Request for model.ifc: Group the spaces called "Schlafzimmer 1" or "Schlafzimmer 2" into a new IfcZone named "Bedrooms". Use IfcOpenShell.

First a look at what the model holds.

```python
import ifcopenshell

model = ifcopenshell.open("model.ifc")
print(model.schema)
seen = {}
for space in model.by_type("IfcSpace"):
    seen[space.LongName] = seen.get(space.LongName, 0) + 1
for name, count in sorted(seen.items(), key=str):
    print(count, "x", name)
print("zones:", [z.Name for z in model.by_type("IfcZone")][:20])
```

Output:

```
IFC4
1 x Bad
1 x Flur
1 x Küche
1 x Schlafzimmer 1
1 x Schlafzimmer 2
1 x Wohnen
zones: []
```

```python
import ifcopenshell
import ifcopenshell.api.group
import ifcopenshell.api.root

model = ifcopenshell.open("model.ifc")

names = {"Schlafzimmer 1", "Schlafzimmer 2"}
spaces = [s for s in model.by_type("IfcSpace") if s.LongName in names]

zone = ifcopenshell.api.root.create_entity(model, ifc_class="IfcZone", name="Bedrooms")
ifcopenshell.api.group.assign_group(model, products=spaces, group=zone)
print(len(spaces), "spaces in", zone.Name)

model.write("model_v2.ifc")
```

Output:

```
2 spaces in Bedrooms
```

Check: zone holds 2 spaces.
